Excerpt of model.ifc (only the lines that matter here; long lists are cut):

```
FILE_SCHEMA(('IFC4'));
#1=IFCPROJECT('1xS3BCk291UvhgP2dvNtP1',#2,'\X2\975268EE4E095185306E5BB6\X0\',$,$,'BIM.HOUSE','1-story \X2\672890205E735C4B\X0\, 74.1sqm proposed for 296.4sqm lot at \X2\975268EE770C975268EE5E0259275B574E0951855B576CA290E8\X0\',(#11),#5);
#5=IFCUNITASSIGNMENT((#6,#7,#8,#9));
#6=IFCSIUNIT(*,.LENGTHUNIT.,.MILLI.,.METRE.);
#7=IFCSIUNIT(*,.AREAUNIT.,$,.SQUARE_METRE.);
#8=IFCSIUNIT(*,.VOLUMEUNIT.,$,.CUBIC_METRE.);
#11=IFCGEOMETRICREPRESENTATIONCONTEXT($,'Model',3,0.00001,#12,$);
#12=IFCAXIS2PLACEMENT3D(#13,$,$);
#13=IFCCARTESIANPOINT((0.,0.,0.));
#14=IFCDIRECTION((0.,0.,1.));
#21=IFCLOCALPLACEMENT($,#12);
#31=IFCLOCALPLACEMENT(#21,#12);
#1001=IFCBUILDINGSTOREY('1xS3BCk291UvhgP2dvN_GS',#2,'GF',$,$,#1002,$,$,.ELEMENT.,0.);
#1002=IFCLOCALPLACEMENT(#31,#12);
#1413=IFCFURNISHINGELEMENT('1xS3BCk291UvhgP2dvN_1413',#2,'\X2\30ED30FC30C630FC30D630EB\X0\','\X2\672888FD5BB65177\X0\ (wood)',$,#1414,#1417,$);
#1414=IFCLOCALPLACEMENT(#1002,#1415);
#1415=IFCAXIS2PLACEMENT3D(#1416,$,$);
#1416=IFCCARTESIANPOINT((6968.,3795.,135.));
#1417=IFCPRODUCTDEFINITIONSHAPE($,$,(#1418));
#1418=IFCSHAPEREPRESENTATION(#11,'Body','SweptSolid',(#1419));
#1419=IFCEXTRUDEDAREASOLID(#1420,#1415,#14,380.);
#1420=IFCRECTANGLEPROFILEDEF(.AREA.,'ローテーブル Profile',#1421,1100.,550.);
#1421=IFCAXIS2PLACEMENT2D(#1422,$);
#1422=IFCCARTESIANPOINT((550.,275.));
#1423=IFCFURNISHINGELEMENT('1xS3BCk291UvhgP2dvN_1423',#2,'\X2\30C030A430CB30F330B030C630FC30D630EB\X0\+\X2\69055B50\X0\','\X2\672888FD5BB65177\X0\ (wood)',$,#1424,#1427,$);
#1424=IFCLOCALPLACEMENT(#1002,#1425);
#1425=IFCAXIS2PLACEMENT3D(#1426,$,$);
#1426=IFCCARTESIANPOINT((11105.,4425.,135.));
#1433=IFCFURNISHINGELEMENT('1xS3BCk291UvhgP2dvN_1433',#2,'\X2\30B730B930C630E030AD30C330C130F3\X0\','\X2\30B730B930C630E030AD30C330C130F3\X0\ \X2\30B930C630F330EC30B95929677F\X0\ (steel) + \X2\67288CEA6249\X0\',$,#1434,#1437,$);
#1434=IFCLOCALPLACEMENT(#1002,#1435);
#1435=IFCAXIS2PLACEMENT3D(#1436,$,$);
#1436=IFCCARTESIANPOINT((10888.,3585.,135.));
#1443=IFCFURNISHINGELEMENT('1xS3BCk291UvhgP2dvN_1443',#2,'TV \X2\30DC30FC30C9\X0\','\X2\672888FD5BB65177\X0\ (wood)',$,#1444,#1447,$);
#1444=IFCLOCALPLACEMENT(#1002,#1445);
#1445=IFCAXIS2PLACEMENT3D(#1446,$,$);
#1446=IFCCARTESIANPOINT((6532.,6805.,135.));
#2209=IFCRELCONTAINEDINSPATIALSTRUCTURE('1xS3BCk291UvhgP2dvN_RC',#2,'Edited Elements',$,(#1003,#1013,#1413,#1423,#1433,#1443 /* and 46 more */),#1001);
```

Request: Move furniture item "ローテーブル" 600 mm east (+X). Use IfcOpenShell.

```python
import ifcopenshell
import ifcopenshell.api.geometry
import ifcopenshell.util.placement
import ifcopenshell.util.unit

model = ifcopenshell.open("model.ifc")
unit_scale = ifcopenshell.util.unit.calculate_unit_scale(model)

item = model.by_guid("1xS3BCk291UvhgP2dvN_1413")
matrix = ifcopenshell.util.placement.get_local_placement(item.ObjectPlacement)
matrix[0, 3] += 0.6 / unit_scale
ifcopenshell.api.geometry.edit_object_placement(model, product=item, matrix=matrix, is_si=False)

print(ifcopenshell.util.placement.get_local_placement(item.ObjectPlacement).round(3) + 0.0)

model.write("model-out.ifc")
```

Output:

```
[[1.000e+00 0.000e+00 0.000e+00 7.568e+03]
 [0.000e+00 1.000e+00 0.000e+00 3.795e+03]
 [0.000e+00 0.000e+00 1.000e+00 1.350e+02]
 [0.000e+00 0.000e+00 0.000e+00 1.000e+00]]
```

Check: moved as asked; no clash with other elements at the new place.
